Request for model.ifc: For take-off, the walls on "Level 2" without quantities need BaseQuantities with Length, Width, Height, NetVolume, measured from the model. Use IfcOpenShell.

First a look at what the model holds.

```python
import ifcopenshell
import ifcopenshell.util.element
import ifcopenshell.util.unit

model = ifcopenshell.open("model.ifc")
print(model.schema)
for unit_type in ("LENGTHUNIT", "AREAUNIT", "VOLUMEUNIT"):
    print(unit_type, ifcopenshell.util.unit.calculate_unit_scale(model, unit_type))
storey = next(s for s in model.by_type("IfcBuildingStorey") if s.Name == "Level 2")
walls = [e for e in ifcopenshell.util.element.get_decomposition(storey) if e.is_a("IfcWall")]
for e in sorted(walls, key=lambda e: e.id()):
    print(e.id(), e.is_a(), e.Name, list(ifcopenshell.util.element.get_psets(e, qtos_only=True)), sep=" | ")
```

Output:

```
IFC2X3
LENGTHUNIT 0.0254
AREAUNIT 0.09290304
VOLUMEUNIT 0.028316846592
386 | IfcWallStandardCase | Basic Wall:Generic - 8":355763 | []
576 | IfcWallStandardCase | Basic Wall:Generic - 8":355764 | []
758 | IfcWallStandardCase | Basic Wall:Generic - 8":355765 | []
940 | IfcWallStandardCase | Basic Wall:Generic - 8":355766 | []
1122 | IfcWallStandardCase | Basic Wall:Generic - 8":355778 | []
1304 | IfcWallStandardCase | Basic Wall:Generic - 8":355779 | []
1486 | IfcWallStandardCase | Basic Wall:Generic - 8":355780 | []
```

```python
import ifcopenshell
import ifcopenshell.api.pset
import ifcopenshell.geom
import ifcopenshell.util.element
import ifcopenshell.util.shape
import ifcopenshell.util.unit

model = ifcopenshell.open("model.ifc")
unit_scale = ifcopenshell.util.unit.calculate_unit_scale(model)
volume_scale = ifcopenshell.util.unit.calculate_unit_scale(model, "VOLUMEUNIT")
settings = ifcopenshell.geom.settings()

storey = next(s for s in model.by_type("IfcBuildingStorey") if s.Name == "Level 2")
walls = [e for e in ifcopenshell.util.element.get_decomposition(storey) if e.is_a("IfcWall")]

for e in sorted(walls, key=lambda e: e.id()):
    if ifcopenshell.util.element.get_psets(e, qtos_only=True, should_inherit=False):
        continue
    # Geometry comes back in metres, in the element's own axes.
    shape = ifcopenshell.geom.create_shape(settings, e)
    values = {
        "Length": ifcopenshell.util.shape.get_x(shape.geometry) / unit_scale,
        "Width": ifcopenshell.util.shape.get_y(shape.geometry) / unit_scale,
        "Height": ifcopenshell.util.shape.get_z(shape.geometry) / unit_scale,
        "NetVolume": ifcopenshell.util.shape.get_volume(shape.geometry) / volume_scale,
    }
    qto = ifcopenshell.api.pset.add_qto(model, product=e, name="BaseQuantities")
    ifcopenshell.api.pset.edit_qto(model, qto=qto, properties=values)
    print(e.id(), {k: round(v, 3) for k, v in values.items()})

model.write("model_v2.ifc")
```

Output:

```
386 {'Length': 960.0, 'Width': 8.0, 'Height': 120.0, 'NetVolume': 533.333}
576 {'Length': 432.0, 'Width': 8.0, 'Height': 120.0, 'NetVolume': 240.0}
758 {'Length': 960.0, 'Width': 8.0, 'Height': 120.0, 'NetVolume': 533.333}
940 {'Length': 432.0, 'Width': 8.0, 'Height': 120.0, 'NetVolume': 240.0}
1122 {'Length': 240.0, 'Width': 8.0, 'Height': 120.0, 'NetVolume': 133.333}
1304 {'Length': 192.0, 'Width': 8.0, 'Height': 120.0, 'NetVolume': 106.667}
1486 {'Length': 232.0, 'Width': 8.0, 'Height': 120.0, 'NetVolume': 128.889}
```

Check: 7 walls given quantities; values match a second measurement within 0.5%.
